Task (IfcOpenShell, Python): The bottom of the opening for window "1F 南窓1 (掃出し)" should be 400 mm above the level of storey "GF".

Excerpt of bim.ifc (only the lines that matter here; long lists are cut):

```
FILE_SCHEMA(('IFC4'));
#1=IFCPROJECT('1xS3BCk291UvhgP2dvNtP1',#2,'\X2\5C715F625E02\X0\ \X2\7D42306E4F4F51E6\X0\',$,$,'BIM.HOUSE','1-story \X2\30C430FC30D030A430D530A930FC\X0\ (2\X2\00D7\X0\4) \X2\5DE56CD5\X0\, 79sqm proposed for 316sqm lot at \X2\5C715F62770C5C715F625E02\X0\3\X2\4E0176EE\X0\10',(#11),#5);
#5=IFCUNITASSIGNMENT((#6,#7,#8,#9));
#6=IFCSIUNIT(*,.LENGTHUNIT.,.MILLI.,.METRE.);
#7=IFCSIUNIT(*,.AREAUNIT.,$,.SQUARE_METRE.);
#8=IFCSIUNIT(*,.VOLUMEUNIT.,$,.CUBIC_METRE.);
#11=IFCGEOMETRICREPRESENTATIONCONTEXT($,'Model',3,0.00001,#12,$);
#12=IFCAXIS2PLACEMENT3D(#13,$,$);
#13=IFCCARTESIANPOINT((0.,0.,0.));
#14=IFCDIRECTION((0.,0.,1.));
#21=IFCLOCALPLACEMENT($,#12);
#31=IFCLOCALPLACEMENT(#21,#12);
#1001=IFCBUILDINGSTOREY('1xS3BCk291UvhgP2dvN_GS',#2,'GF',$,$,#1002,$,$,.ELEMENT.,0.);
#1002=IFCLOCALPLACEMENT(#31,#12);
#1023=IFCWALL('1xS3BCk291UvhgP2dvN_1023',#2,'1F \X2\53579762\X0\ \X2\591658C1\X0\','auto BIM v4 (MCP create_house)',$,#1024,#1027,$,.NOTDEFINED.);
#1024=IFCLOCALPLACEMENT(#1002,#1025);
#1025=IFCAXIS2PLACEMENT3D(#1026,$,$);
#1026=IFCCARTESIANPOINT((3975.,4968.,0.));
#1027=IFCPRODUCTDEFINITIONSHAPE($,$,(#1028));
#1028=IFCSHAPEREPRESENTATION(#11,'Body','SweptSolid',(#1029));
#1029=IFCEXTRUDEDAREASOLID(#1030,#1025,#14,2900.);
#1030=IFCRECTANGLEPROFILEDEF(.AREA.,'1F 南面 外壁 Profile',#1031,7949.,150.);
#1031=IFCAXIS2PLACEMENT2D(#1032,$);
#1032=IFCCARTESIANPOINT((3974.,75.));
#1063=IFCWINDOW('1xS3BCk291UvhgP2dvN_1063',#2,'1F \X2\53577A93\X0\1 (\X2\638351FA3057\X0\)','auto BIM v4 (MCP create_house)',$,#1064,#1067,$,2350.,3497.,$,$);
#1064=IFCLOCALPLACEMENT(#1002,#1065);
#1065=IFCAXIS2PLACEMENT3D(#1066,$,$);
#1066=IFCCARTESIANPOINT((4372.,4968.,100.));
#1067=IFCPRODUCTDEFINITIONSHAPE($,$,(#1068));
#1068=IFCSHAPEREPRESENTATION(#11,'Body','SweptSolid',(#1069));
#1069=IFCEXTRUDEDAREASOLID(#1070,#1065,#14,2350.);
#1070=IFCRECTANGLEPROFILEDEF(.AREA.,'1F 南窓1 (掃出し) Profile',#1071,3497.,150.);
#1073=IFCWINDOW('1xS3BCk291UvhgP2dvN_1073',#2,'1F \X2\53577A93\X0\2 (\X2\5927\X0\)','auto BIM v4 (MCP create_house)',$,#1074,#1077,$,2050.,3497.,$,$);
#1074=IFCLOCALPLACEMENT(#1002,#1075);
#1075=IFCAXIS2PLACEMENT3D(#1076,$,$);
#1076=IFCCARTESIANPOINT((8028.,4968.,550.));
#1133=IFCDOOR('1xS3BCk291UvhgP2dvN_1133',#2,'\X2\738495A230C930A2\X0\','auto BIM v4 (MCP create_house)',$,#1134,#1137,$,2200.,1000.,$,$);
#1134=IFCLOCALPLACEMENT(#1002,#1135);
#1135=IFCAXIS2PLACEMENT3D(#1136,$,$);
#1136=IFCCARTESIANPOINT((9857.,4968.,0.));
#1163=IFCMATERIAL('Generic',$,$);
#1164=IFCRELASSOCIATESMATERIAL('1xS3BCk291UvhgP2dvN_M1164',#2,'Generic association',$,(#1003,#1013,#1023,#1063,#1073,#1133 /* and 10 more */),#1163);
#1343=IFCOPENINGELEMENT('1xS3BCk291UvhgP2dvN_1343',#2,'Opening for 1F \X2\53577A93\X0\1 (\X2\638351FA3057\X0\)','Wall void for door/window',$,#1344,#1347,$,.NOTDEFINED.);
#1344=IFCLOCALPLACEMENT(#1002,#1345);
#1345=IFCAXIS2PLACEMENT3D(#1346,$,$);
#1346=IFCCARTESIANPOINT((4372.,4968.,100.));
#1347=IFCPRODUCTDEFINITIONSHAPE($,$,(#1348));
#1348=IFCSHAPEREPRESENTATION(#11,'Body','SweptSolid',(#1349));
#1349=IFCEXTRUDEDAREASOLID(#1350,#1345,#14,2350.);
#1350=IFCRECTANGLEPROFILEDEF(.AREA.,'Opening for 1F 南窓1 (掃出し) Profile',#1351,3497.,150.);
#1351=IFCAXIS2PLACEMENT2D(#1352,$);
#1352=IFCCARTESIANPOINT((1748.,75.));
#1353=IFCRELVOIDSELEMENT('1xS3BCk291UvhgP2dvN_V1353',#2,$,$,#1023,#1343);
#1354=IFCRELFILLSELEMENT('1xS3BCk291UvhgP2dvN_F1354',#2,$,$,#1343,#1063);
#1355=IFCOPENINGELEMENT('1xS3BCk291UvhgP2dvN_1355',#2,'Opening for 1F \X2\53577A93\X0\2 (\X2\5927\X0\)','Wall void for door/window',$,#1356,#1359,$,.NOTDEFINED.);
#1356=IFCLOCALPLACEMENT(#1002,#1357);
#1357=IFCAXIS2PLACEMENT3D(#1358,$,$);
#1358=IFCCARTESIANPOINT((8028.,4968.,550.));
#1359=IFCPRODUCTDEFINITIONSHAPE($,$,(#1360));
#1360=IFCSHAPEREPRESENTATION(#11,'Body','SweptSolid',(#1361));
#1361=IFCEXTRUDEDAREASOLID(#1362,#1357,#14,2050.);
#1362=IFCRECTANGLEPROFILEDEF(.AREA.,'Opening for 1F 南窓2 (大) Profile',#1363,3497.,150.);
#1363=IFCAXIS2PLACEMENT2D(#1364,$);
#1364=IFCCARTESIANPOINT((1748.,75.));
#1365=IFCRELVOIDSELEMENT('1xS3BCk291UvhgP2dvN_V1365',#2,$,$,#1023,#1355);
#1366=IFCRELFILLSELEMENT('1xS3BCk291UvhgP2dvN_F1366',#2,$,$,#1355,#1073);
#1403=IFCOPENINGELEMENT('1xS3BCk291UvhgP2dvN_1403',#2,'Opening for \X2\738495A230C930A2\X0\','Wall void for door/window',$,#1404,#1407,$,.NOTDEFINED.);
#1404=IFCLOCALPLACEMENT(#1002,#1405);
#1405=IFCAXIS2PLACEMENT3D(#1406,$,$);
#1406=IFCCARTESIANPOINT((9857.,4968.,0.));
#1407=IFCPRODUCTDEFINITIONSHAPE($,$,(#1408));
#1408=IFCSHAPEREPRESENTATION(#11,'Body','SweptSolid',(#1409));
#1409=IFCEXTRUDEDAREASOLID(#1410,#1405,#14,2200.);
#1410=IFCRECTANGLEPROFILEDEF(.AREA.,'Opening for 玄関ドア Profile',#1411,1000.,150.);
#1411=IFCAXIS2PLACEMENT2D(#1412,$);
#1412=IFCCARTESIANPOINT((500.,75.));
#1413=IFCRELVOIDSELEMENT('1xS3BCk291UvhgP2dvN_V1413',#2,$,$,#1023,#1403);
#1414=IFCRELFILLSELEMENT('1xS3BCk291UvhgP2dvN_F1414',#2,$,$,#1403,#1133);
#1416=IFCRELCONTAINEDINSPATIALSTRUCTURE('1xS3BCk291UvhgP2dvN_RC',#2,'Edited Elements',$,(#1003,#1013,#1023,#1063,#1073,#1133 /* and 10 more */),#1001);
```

```python
import numpy as np
import ifcopenshell
import ifcopenshell.api.geometry
import ifcopenshell.geom
import ifcopenshell.util.element
import ifcopenshell.util.placement
import ifcopenshell.util.shape
import ifcopenshell.util.unit

model = ifcopenshell.open("bim.ifc")
unit_scale = ifcopenshell.util.unit.calculate_unit_scale(model)

window = model.by_guid("1xS3BCk291UvhgP2dvN_1063")
opening = window.FillsVoids[0].RelatingOpeningElement
storey = ifcopenshell.util.element.get_container(window, ifc_class="IfcBuildingStorey")
level = ifcopenshell.util.placement.get_local_placement(storey.ObjectPlacement)[2, 3]

# The opening's origin need not be at the sill, so measure its lowest point.
shape = ifcopenshell.geom.create_shape(ifcopenshell.geom.settings(), opening)
bottom = ifcopenshell.util.shape.get_shape_bottom_elevation(shape, shape.geometry) / unit_scale
dz = level + 0.4 / unit_scale - bottom

shift = np.array([0.0, 0.0, dz])
# The window is not placed relative to its opening, so move both.
for product in (opening, window):
    matrix = ifcopenshell.util.placement.get_local_placement(product.ObjectPlacement)
    matrix[:3, 3] += shift
    ifcopenshell.api.geometry.edit_object_placement(model, product=product, matrix=matrix, is_si=False)

print(f"moved by {dz * unit_scale:+.3f} m")

model.write("bim_v2.ifc")
```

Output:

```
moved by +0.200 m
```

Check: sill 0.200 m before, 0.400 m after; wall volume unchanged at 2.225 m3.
